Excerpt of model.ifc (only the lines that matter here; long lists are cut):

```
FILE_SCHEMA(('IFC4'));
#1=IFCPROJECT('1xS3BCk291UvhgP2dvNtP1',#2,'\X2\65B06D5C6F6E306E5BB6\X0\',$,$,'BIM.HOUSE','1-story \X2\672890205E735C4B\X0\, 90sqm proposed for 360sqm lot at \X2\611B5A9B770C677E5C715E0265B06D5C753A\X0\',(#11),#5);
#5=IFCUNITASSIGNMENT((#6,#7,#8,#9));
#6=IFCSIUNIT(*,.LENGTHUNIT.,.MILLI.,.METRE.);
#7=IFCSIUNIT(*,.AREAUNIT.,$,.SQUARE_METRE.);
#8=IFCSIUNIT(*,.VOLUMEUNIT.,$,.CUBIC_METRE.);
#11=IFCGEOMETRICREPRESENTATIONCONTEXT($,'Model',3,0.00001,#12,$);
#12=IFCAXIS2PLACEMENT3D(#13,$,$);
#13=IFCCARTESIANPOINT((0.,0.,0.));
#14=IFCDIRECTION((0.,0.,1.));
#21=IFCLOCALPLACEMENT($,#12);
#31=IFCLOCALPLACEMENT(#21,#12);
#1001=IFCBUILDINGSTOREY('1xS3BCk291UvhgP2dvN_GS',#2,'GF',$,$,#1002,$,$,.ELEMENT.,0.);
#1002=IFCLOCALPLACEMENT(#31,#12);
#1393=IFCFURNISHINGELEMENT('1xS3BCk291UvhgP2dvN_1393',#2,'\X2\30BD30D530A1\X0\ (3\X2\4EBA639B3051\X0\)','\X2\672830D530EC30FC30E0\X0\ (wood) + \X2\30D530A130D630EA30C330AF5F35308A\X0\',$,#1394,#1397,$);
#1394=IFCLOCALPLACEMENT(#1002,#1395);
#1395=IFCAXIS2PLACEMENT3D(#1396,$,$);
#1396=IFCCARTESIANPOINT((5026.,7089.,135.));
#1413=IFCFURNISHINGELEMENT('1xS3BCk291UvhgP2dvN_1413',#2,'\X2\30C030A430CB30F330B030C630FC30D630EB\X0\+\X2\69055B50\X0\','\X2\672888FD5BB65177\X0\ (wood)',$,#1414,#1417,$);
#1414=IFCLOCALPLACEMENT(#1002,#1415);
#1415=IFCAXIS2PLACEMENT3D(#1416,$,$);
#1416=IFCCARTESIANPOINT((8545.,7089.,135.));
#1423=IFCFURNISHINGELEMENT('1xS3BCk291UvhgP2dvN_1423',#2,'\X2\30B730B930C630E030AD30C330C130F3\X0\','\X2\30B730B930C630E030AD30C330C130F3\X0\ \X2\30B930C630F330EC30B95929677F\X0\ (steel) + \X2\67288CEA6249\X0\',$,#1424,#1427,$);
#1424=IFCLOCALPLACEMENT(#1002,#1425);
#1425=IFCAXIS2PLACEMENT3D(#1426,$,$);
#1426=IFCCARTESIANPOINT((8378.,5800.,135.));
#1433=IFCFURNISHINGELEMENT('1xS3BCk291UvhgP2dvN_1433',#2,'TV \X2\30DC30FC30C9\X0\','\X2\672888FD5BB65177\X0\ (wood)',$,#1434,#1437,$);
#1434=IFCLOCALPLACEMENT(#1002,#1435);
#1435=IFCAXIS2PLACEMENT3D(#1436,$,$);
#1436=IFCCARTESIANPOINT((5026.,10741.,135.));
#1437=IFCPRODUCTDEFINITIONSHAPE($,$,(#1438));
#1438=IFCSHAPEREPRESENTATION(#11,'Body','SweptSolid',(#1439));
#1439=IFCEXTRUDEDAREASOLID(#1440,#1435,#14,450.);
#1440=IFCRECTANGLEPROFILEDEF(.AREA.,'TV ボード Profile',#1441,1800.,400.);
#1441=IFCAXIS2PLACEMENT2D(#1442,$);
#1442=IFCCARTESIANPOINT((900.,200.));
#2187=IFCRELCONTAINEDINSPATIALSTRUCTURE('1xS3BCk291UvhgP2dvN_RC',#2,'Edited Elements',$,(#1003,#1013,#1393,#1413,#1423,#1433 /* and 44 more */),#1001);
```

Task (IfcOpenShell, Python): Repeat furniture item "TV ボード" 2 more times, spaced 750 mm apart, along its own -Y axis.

```python
import ifcopenshell
import ifcopenshell.api.geometry
import ifcopenshell.api.root
import ifcopenshell.util.element
import ifcopenshell.util.placement
import ifcopenshell.util.unit

model = ifcopenshell.open("model.ifc")
unit_scale = ifcopenshell.util.unit.calculate_unit_scale(model)


def reuse_history(source, copy):
    """copy_class also copies each property set's owner history, people and application; keep the originals."""
    for rel in copy.IsDefinedBy:
        if rel.is_a("IfcRelDefinesByProperties") and (history := rel.RelatingPropertyDefinition.OwnerHistory):
            rel.RelatingPropertyDefinition.OwnerHistory = source.OwnerHistory
            ifcopenshell.util.element.remove_deep2(model, history)


source = model.by_guid("1xS3BCk291UvhgP2dvN_1433")
base = ifcopenshell.util.placement.get_local_placement(source.ObjectPlacement)
step = -base[:3, 1] * 0.75 / unit_scale

for i in range(1, 3):
    copy = ifcopenshell.api.root.copy_class(model, product=source)
    copy.Representation = ifcopenshell.util.element.copy_deep(
        model, source.Representation, exclude=["IfcGeometricRepresentationContext", "IfcRepresentationMap"]
    )
    reuse_history(source, copy)
    matrix = base.copy()
    matrix[:3, 3] += i * step
    print("added at", matrix[:3, 3].round(3) + 0.0)
    ifcopenshell.api.geometry.edit_object_placement(model, product=copy, matrix=matrix, is_si=False)

model.write("model_rev.ifc")
```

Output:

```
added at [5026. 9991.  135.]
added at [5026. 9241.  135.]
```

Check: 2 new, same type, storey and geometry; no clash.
